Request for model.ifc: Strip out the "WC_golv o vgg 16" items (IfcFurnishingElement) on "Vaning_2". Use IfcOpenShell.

First a look at what the model holds.

```python
import ifcopenshell
import ifcopenshell.util.element

model = ifcopenshell.open("model.ifc")
print(model.schema)
storey = next(s for s in model.by_type("IfcBuildingStorey") if s.Name == "Vaning_2")
furniture = [e for e in ifcopenshell.util.element.get_decomposition(storey) if e.is_a("IfcFurnishingElement")]
seen = {}
for e in furniture:
    element_type = ifcopenshell.util.element.get_type(e)
    name = element_type.Name if element_type not in (None, e) else None
    seen[name] = seen.get(name, 0) + 1
for name, count in sorted(seen.items(), key=str):
    print(count, "x", name)
```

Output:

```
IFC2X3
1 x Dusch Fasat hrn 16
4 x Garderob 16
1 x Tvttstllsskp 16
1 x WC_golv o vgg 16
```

```python
import ifcopenshell
import ifcopenshell.api.root
import ifcopenshell.util.element

model = ifcopenshell.open("model.ifc")

storey = next(s for s in model.by_type("IfcBuildingStorey") if s.Name == "Vaning_2")
furniture = [e for e in ifcopenshell.util.element.get_decomposition(storey) if e.is_a("IfcFurnishingElement")]
targets = [e for e in furniture if (t := ifcopenshell.util.element.get_type(e)) not in (None, e) and t.Name == 'WC_golv o v\x8agg 16']

for e in targets:
    ifcopenshell.api.root.remove_product(model, product=e)
print(len(targets), "removed")

model.write("model-out.ifc")
```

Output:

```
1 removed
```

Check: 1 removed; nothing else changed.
